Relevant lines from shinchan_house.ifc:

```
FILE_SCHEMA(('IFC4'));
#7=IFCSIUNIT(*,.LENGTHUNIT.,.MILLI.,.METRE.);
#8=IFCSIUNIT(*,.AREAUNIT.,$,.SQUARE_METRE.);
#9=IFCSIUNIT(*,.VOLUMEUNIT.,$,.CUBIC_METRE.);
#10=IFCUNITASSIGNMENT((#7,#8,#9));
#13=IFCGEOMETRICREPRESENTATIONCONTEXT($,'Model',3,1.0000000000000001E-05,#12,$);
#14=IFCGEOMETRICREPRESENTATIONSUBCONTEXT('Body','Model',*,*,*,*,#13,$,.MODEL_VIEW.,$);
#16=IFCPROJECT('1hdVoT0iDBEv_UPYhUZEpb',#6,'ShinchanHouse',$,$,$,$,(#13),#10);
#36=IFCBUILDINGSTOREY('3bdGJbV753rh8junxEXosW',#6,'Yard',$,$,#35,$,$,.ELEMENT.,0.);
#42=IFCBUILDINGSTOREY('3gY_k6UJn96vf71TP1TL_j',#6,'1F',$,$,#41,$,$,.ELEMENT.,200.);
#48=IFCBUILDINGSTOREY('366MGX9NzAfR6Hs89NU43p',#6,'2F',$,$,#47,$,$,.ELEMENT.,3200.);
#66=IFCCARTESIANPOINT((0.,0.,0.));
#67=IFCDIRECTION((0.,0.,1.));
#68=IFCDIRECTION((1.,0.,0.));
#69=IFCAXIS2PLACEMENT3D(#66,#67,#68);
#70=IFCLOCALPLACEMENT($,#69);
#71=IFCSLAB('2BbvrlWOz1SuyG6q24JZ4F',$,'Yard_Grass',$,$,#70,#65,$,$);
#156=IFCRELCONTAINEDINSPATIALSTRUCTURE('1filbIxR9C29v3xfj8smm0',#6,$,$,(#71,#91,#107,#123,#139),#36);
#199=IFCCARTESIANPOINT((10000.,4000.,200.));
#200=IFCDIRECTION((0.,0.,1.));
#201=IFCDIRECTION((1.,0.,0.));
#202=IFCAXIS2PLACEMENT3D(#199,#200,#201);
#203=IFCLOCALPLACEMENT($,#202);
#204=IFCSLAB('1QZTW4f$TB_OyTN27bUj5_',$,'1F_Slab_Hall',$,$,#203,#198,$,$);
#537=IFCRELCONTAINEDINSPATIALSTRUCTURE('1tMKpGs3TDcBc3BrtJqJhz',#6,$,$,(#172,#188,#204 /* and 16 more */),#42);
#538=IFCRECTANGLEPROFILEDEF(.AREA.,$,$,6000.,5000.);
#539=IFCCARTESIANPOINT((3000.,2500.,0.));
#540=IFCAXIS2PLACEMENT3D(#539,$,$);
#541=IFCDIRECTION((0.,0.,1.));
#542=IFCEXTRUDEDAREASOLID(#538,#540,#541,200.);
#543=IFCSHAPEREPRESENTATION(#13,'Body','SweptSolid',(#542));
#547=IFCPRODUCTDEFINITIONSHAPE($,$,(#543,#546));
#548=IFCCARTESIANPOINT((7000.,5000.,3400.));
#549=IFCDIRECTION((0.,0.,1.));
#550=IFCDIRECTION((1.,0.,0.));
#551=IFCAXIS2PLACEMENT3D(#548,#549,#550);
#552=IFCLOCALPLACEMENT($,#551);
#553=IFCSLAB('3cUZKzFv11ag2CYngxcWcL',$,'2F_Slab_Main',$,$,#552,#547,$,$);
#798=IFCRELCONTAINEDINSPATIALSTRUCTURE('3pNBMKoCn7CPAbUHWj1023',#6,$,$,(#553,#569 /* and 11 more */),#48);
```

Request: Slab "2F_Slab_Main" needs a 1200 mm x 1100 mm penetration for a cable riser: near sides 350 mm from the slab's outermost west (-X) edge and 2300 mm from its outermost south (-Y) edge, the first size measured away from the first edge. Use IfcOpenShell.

```python
import numpy as np
import ifcopenshell
import ifcopenshell.api.feature
import ifcopenshell.api.geometry
import ifcopenshell.api.root
import ifcopenshell.geom
import ifcopenshell.util.placement
import ifcopenshell.util.representation
import ifcopenshell.util.shape
import ifcopenshell.util.unit

model = ifcopenshell.open("shinchan_house.ifc")
unit_scale = ifcopenshell.util.unit.calculate_unit_scale(model)
settings = ifcopenshell.geom.settings()


def volume(element):
    """Net volume in cubic metres, openings subtracted."""
    shape = ifcopenshell.geom.create_shape(settings, element)
    return ifcopenshell.util.shape.get_volume(shape.geometry)


slab = model.by_guid("3cUZKzFv11ag2CYngxcWcL")
before = volume(slab)

# Extent in the slab's own axes, in metres. The edges named are its -X and -Y sides.
slab_shape = ifcopenshell.geom.create_shape(settings, slab)
vertices = ifcopenshell.util.shape.get_vertices(slab_shape.geometry)
x_min, y_min, bottom = vertices.min(axis=0)
top = vertices[:, 2].max()

opening = ifcopenshell.api.root.create_entity(model, ifc_class="IfcOpeningElement", name="Cable riser opening", predefined_type="OPENING")
context = ifcopenshell.util.representation.get_context(model, "Model", "Body", "MODEL_VIEW")
width, depth = 1.2, 1.1
outline = [(0.0, 0.0), (width, 0.0), (width, depth), (0.0, depth), (0.0, 0.0)]
# Overshoot both faces by 50 mm so the cut is clean.
shape = ifcopenshell.api.geometry.add_slab_representation(
    model, context=context, depth=top - bottom + 0.1, polyline=outline
)
ifcopenshell.api.geometry.assign_representation(model, product=opening, representation=shape)

matrix = ifcopenshell.util.placement.get_local_placement(slab.ObjectPlacement)
matrix[:, 3] = matrix @ np.append(np.array([x_min + 0.35, y_min + 2.3, bottom - 0.05]) / unit_scale, 1.0)
ifcopenshell.api.geometry.edit_object_placement(model, product=opening, matrix=matrix, is_si=False)
ifcopenshell.api.feature.add_feature(model, feature=opening, element=slab)

after = volume(slab)

print(f"slab volume {before:.3f} -> {after:.3f} m3")

model.write("shinchan_house_edited.ifc")
```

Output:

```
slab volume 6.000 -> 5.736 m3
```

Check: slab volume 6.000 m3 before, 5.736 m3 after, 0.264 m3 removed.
